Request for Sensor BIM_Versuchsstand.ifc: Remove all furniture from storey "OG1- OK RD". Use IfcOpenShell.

First a look at what the model holds.

```python
import ifcopenshell
import ifcopenshell.util.element

model = ifcopenshell.open("Sensor BIM_Versuchsstand.ifc")
print(model.schema)
storey = next(s for s in model.by_type("IfcBuildingStorey") if s.Name == "OG1- OK RD")
furniture = [e for e in ifcopenshell.util.element.get_decomposition(storey) if e.is_a("IfcFurnishingElement")]
seen = {}
for e in furniture:
    element_type = ifcopenshell.util.element.get_type(e)
    name = element_type.Name if element_type not in (None, e) else None
    seen[name] = seen.get(name, 0) + 1
for name, count in sorted(seen.items(), key=str):
    print(count, "x", name)
```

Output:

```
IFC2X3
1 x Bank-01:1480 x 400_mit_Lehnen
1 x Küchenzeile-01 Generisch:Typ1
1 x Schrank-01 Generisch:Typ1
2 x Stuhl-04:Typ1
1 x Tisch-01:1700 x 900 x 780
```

```python
import ifcopenshell
import ifcopenshell.api.root
import ifcopenshell.util.element

model = ifcopenshell.open("Sensor BIM_Versuchsstand.ifc")

storey = next(s for s in model.by_type("IfcBuildingStorey") if s.Name == "OG1- OK RD")
furniture = [e for e in ifcopenshell.util.element.get_decomposition(storey) if e.is_a("IfcFurnishingElement")]

for e in furniture:
    ifcopenshell.api.root.remove_product(model, product=e)
print(len(furniture), "removed")

model.write("Sensor BIM_Versuchsstand_edited.ifc")
```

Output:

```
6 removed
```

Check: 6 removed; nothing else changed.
